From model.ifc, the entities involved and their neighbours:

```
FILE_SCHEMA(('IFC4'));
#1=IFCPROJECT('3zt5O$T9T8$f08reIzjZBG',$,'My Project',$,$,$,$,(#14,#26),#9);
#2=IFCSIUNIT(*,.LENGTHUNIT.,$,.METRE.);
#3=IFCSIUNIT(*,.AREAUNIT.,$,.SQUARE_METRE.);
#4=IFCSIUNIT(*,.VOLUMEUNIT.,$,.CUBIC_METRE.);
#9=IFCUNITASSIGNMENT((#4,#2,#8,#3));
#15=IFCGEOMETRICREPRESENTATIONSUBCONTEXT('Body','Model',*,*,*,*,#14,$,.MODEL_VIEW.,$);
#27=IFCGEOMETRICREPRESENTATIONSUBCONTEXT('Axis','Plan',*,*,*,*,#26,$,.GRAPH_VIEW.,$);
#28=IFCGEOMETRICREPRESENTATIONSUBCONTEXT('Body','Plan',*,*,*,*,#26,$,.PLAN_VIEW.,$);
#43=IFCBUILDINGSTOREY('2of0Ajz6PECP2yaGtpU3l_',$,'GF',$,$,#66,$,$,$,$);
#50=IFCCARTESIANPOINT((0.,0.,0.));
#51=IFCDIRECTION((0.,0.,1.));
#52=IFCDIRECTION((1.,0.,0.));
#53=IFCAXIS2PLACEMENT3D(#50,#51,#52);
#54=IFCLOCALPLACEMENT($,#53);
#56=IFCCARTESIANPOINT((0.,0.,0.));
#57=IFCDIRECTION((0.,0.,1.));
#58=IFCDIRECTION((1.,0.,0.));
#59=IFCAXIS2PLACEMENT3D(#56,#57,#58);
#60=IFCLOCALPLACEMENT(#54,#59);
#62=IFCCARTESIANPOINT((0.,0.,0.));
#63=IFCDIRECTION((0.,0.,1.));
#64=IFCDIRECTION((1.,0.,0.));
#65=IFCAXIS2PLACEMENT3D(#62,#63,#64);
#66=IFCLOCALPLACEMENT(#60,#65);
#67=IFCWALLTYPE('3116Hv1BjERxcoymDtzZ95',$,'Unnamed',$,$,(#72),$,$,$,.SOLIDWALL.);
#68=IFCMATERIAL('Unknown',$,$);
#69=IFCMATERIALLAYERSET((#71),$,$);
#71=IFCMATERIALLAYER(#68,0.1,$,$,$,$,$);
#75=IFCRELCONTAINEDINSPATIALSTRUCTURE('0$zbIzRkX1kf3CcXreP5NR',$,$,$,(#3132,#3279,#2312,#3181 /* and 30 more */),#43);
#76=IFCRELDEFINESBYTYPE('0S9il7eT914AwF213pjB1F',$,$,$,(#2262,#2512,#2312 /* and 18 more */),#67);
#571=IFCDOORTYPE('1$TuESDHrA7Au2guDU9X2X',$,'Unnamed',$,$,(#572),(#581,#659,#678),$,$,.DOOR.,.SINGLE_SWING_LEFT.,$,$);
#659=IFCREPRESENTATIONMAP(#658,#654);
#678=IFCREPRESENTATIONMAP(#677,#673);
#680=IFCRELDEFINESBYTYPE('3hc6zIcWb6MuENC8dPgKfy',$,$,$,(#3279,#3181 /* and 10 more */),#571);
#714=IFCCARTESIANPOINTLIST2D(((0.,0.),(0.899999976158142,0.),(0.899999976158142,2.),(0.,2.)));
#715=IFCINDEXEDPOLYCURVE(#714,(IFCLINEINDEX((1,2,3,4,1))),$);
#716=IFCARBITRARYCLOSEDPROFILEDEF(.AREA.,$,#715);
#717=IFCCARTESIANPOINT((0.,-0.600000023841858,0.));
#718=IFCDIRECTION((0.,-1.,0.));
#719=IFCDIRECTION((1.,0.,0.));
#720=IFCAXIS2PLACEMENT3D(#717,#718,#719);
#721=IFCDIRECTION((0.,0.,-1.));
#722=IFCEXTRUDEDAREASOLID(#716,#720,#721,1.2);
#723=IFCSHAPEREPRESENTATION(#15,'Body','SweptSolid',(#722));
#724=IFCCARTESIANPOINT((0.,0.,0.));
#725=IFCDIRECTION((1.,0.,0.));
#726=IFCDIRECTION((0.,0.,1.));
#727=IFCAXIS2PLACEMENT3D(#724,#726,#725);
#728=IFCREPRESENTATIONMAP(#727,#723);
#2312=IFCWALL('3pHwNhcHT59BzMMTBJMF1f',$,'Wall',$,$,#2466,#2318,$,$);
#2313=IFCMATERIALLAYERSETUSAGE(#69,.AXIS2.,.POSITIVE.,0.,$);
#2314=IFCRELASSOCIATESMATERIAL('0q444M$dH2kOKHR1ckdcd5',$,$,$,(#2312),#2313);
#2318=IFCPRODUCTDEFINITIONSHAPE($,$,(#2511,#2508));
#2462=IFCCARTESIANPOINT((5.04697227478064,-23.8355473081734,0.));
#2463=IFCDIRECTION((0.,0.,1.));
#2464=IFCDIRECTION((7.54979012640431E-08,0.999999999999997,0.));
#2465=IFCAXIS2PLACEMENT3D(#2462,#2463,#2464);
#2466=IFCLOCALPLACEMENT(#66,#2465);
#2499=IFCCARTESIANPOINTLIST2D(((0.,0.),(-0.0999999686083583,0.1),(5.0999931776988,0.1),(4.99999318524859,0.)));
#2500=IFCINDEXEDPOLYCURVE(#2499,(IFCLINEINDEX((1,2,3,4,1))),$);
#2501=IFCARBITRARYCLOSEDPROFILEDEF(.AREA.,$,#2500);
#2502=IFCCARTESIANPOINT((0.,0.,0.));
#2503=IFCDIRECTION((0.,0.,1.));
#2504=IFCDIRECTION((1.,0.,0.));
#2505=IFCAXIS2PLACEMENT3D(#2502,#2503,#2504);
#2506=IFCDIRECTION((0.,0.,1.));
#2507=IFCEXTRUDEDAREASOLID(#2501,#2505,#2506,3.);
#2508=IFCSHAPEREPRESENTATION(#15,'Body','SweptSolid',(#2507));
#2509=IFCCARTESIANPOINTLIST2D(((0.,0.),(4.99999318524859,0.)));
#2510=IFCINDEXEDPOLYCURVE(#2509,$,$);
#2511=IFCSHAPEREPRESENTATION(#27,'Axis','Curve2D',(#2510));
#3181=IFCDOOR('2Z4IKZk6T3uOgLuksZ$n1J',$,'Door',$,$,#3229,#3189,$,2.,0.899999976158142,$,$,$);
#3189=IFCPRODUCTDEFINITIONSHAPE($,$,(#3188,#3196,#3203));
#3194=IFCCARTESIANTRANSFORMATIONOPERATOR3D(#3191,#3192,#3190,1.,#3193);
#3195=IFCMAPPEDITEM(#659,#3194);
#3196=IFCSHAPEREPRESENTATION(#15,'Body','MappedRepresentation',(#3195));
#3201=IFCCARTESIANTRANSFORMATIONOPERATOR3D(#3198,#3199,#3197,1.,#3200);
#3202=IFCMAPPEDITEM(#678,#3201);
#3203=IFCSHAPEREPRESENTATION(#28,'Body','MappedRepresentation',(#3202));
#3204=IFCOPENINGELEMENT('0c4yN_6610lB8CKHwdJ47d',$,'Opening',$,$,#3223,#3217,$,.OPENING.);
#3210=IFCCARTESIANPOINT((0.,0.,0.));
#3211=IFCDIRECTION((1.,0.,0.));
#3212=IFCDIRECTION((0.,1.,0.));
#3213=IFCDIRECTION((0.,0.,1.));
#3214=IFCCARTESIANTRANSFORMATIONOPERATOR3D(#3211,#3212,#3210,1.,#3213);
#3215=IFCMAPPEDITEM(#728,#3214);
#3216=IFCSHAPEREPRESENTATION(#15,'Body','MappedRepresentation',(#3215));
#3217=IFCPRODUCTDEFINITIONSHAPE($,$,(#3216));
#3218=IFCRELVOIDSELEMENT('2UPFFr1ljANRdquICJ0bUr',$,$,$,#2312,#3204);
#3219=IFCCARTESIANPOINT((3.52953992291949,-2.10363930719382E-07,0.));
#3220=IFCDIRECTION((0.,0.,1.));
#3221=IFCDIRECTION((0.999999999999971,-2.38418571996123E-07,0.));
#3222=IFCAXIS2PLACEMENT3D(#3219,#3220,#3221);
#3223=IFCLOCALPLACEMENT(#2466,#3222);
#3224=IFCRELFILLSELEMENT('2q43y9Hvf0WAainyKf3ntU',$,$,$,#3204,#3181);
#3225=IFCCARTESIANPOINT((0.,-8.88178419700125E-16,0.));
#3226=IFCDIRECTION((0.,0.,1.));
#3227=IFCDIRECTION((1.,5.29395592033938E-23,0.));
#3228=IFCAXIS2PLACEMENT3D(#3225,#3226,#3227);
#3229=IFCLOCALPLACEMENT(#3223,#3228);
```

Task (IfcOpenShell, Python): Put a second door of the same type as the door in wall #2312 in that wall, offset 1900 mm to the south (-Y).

```python
import ifcopenshell
import ifcopenshell.api.feature
import ifcopenshell.api.geometry
import ifcopenshell.api.root
import ifcopenshell.geom
import ifcopenshell.util.element
import ifcopenshell.util.placement
import ifcopenshell.util.shape

model = ifcopenshell.open("model.ifc")
settings = ifcopenshell.geom.settings()


def volume(element):
    """Net volume in cubic metres, openings subtracted."""
    shape = ifcopenshell.geom.create_shape(settings, element)
    return ifcopenshell.util.shape.get_volume(shape.geometry)


door = model.by_guid("2Z4IKZk6T3uOgLuksZ$n1J")
opening = door.FillsVoids[0].RelatingOpeningElement
wall = opening.VoidsElements[0].RelatingBuildingElement
before = volume(wall)
shift = ifcopenshell.util.placement.get_local_placement(wall.ObjectPlacement)[:3, 0] * -1.9

# copy_class copies the void relationship, type, container and properties, but no geometry.
new_opening = ifcopenshell.api.root.copy_class(model, product=opening)
new_opening.Representation = ifcopenshell.util.element.copy_deep(
    model, opening.Representation, exclude=["IfcGeometricRepresentationContext", "IfcRepresentationMap"]
)
new_door = ifcopenshell.api.root.copy_class(model, product=door)
new_door.Representation = ifcopenshell.util.element.copy_deep(
    model, door.Representation, exclude=["IfcGeometricRepresentationContext", "IfcRepresentationMap"]
)
ifcopenshell.api.feature.add_filling(model, opening=new_opening, element=new_door)

for old, new in ((opening, new_opening), (door, new_door)):
    matrix = ifcopenshell.util.placement.get_local_placement(old.ObjectPlacement)
    matrix[:3, 3] += shift
    ifcopenshell.api.geometry.edit_object_placement(model, product=new, matrix=matrix, is_si=False)

after = volume(wall)

print(f"wall volume {before:.3f} -> {after:.3f} m3")

model.write("model-out.ifc")
```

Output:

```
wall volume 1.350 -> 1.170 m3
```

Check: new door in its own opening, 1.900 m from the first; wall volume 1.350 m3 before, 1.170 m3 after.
